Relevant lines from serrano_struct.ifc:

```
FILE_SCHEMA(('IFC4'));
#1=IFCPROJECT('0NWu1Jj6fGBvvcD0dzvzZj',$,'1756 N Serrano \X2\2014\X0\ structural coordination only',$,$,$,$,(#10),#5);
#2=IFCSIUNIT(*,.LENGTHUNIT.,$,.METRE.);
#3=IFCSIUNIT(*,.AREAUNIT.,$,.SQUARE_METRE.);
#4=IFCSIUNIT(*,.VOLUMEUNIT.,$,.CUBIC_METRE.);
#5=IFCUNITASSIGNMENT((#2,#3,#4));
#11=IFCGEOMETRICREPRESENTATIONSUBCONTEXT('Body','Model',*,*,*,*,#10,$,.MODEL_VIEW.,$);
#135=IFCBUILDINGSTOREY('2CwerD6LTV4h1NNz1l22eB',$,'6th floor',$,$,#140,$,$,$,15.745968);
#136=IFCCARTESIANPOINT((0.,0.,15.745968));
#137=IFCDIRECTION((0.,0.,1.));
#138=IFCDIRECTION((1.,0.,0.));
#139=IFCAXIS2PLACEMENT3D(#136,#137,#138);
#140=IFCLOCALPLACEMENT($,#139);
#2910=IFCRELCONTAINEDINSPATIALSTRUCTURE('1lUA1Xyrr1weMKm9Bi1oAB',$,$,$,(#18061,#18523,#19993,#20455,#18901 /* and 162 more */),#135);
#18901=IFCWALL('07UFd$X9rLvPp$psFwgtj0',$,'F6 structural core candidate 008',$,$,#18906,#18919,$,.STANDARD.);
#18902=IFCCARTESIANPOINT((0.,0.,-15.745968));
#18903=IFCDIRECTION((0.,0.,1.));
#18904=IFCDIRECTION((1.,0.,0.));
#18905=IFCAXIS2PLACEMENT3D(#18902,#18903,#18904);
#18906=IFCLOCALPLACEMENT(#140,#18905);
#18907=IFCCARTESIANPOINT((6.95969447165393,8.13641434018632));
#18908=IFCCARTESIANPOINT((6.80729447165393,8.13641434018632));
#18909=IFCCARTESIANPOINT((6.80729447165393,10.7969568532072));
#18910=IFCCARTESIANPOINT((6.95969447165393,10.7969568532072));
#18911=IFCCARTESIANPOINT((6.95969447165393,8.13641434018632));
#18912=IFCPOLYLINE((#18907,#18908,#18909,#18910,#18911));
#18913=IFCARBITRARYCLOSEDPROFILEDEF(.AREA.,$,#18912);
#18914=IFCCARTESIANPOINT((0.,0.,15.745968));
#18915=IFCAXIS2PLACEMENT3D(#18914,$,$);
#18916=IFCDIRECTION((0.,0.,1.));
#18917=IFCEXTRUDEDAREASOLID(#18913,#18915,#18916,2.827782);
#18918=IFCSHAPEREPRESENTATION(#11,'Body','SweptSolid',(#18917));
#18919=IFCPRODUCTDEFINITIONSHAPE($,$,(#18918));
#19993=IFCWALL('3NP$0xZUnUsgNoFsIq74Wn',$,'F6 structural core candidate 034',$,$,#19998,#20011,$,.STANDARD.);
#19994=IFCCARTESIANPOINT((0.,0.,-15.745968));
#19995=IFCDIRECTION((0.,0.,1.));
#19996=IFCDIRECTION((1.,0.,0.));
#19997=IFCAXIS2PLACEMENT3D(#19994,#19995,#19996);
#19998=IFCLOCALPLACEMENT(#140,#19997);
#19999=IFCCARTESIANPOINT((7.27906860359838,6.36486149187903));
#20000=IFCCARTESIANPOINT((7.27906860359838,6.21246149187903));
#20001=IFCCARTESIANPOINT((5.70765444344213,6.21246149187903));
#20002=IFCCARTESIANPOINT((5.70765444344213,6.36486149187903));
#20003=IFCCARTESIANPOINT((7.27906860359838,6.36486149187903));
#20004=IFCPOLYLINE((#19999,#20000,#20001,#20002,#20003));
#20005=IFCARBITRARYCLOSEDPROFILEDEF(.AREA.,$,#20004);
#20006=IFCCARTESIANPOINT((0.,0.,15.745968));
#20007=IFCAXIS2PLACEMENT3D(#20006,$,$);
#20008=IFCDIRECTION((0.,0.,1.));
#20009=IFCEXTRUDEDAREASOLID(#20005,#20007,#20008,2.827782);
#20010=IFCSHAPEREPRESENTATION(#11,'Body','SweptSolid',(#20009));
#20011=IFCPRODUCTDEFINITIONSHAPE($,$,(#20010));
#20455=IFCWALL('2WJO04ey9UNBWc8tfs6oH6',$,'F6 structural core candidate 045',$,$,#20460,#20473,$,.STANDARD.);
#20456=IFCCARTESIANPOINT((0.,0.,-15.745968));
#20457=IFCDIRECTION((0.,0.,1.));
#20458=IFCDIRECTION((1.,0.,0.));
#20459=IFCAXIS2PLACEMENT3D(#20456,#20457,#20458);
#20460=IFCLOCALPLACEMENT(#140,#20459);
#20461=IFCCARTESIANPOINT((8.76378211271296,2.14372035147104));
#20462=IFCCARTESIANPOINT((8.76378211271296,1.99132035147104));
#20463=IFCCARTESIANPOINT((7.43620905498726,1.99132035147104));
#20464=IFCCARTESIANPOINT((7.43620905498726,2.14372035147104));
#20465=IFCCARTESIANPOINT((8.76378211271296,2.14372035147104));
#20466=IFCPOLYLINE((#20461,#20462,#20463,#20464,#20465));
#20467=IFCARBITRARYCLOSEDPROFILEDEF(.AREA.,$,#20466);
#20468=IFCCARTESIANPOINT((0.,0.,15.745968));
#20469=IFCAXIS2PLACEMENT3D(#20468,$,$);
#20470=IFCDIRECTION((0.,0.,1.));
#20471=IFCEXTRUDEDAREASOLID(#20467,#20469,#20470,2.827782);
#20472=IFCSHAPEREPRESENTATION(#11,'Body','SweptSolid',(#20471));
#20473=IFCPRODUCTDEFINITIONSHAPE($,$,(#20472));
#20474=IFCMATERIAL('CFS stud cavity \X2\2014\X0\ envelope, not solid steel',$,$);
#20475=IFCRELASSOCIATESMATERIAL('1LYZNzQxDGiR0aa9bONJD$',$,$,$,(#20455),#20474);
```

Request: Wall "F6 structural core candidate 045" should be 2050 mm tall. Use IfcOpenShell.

```python
import ifcopenshell
import ifcopenshell.geom
import ifcopenshell.util.representation
import ifcopenshell.util.shape
import ifcopenshell.util.unit

model = ifcopenshell.open("serrano_struct.ifc")
unit_scale = ifcopenshell.util.unit.calculate_unit_scale(model)
settings = ifcopenshell.geom.settings()


def volume(element):
    """Net volume in cubic metres, openings subtracted."""
    shape = ifcopenshell.geom.create_shape(settings, element)
    return ifcopenshell.util.shape.get_volume(shape.geometry)


wall = model.by_guid("2WJO04ey9UNBWc8tfs6oH6")
before = volume(wall)

body = ifcopenshell.util.representation.get_representation(wall, "Model", "Body")
solid = body.Items[0]
old_height = solid.Depth
solid.Depth = 2.05 / unit_scale
after = volume(wall)

print(f"height {old_height:g} -> {solid.Depth:g}, volume {before:.3f} -> {after:.3f} m3")

model.write("serrano_struct_rev.ifc")
```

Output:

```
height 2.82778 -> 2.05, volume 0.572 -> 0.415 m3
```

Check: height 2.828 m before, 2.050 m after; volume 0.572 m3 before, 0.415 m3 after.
